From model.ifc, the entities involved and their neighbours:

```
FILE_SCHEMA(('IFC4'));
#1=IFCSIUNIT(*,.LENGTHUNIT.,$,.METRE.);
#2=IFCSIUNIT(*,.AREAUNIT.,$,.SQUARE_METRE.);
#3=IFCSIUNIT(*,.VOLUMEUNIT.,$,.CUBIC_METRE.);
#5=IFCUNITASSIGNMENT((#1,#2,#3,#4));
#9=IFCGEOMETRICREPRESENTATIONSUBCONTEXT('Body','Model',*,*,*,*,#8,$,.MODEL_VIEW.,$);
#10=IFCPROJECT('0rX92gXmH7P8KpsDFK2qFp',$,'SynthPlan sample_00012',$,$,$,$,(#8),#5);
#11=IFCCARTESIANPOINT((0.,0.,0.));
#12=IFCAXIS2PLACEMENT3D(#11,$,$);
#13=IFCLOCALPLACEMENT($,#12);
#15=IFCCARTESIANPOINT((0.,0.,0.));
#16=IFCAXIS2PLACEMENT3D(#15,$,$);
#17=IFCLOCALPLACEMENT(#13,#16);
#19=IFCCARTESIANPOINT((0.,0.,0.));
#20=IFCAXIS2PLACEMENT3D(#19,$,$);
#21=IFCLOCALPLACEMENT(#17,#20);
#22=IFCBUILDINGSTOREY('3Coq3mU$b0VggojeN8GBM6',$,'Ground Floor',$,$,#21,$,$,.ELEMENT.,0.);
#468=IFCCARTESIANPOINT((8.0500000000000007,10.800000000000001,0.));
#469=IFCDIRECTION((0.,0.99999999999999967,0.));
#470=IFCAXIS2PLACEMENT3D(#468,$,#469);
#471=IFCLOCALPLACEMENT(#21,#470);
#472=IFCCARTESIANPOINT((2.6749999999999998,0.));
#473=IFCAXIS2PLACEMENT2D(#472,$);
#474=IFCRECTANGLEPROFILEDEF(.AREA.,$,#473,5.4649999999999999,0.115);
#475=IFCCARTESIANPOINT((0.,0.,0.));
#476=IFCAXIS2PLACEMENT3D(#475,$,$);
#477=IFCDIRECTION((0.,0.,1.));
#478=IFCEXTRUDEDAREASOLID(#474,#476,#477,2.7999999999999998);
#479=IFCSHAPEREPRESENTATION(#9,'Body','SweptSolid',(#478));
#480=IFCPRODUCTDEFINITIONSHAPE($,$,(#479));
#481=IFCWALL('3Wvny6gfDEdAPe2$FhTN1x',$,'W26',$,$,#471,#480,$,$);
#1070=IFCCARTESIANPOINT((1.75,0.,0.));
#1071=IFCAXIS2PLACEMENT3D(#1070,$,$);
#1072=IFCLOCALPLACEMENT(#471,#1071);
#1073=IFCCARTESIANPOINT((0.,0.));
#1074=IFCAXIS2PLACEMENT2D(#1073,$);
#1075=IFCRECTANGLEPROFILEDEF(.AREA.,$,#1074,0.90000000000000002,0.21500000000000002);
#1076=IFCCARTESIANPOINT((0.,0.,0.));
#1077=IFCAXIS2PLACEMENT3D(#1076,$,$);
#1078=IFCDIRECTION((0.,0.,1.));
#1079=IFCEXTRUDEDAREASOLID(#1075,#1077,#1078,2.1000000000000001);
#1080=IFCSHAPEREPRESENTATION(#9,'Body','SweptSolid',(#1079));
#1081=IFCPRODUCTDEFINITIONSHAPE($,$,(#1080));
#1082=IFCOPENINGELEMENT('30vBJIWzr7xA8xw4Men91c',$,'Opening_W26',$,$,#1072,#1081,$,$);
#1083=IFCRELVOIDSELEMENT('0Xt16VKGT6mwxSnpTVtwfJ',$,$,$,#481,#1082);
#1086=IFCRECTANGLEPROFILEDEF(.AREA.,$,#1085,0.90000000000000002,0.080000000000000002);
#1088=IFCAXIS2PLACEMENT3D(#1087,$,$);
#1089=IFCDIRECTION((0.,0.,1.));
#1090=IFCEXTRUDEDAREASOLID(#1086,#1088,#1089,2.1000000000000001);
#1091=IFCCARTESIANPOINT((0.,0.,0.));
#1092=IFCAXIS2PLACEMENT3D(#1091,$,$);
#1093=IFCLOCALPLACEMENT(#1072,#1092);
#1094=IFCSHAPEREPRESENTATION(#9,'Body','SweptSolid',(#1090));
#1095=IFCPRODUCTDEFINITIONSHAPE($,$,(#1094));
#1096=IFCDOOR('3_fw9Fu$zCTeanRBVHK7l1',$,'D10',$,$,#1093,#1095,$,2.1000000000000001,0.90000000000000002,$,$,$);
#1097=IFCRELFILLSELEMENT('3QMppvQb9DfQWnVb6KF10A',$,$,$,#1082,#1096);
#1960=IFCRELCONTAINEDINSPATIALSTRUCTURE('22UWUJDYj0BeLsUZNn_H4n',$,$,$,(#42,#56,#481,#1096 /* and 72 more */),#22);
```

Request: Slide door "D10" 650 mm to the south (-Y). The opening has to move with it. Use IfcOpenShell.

```python
import ifcopenshell
import ifcopenshell.api.geometry
import ifcopenshell.util.placement
import ifcopenshell.util.unit

model = ifcopenshell.open("model.ifc")
unit_scale = ifcopenshell.util.unit.calculate_unit_scale(model)

door = model.by_id(1096)
opening = door.FillsVoids[0].RelatingOpeningElement
wall = opening.VoidsElements[0].RelatingBuildingElement

wall_matrix = ifcopenshell.util.placement.get_local_placement(wall.ObjectPlacement)
shift = wall_matrix[:3, 0] * -0.65 / unit_scale
before = ifcopenshell.util.placement.get_local_placement(door.ObjectPlacement)[:3, 3].copy()

# The door is placed relative to its opening, so it follows when the opening moves.
matrix = ifcopenshell.util.placement.get_local_placement(opening.ObjectPlacement)
matrix[:3, 3] += shift
ifcopenshell.api.geometry.edit_object_placement(
    model, product=opening, matrix=matrix, is_si=False, should_transform_children=True
)

after = ifcopenshell.util.placement.get_local_placement(door.ObjectPlacement)[:3, 3]
print("door moved by", (after - before).round(3) + 0.0)

model.write("model_v2.ifc")
```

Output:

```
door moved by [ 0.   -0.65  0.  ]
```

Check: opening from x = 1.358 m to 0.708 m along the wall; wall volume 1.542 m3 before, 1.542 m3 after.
